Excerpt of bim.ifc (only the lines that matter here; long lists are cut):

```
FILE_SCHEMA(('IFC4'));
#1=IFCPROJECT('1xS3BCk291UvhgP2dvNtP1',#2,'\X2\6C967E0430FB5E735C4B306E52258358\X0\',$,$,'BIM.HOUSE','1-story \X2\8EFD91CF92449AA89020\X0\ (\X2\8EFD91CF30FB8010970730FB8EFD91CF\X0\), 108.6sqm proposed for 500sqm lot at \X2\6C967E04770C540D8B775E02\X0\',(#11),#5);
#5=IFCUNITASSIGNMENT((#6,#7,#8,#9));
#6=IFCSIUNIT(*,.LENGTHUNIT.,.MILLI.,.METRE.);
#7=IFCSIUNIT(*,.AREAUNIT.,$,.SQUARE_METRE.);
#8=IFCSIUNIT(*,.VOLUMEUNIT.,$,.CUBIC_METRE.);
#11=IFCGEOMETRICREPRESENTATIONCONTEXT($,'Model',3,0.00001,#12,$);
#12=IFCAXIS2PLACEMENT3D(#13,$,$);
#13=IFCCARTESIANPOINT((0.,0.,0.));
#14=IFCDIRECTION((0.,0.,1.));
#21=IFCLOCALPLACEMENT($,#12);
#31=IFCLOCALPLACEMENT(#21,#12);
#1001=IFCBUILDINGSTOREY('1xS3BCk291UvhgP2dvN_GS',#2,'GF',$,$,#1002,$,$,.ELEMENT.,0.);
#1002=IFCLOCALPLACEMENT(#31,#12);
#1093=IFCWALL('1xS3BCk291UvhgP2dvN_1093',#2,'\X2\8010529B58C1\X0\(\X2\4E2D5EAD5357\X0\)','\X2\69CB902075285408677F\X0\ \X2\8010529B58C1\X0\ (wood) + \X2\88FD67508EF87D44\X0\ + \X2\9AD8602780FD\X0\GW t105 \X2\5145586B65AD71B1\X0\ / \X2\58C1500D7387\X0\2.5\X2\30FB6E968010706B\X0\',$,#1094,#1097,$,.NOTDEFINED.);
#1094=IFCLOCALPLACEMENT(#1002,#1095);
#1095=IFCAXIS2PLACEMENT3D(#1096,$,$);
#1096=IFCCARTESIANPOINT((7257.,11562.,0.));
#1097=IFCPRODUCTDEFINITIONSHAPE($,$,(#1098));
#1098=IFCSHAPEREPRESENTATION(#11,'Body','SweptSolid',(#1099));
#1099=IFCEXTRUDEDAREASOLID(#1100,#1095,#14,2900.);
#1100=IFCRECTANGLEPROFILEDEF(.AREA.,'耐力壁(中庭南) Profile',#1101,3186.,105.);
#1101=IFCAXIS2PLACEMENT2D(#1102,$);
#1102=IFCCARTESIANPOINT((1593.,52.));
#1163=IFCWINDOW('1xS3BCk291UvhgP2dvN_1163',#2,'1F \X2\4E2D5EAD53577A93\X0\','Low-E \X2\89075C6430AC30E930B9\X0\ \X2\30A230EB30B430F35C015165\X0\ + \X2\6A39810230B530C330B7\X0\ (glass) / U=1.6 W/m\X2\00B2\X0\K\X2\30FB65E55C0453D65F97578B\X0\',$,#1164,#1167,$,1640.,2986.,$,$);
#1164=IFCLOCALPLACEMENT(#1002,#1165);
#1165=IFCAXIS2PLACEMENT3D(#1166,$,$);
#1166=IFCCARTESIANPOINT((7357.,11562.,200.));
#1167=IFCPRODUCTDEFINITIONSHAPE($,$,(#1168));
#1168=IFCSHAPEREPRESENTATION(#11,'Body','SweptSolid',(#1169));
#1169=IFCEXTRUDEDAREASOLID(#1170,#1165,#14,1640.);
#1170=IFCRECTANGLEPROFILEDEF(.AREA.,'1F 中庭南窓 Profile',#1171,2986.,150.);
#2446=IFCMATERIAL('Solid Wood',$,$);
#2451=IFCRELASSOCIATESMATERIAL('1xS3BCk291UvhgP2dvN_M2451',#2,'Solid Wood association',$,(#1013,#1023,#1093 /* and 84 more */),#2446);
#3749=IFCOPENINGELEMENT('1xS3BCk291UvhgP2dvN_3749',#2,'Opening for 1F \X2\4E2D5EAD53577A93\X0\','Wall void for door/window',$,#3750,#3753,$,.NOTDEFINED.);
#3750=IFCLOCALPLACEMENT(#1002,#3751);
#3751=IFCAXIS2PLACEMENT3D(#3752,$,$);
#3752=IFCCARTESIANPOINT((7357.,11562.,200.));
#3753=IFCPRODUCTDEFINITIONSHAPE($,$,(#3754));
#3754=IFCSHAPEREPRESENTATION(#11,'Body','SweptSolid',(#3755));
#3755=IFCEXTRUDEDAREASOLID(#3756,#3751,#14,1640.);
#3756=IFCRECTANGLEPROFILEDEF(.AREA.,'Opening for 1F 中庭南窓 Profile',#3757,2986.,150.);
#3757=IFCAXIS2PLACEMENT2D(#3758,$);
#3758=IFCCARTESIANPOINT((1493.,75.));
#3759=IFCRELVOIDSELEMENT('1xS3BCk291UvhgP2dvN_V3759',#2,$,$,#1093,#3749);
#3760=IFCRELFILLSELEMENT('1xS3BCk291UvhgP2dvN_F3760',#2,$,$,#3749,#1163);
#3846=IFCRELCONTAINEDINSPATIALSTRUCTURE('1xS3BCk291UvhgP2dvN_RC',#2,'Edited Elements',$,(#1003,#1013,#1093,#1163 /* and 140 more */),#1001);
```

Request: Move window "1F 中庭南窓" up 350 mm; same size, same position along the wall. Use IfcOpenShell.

```python
import numpy as np
import ifcopenshell
import ifcopenshell.api.geometry
import ifcopenshell.util.placement
import ifcopenshell.util.unit

model = ifcopenshell.open("bim.ifc")
unit_scale = ifcopenshell.util.unit.calculate_unit_scale(model)

window = model.by_guid("1xS3BCk291UvhgP2dvN_1163")
opening = window.FillsVoids[0].RelatingOpeningElement
dz = 0.35 / unit_scale

shift = np.array([0.0, 0.0, dz])
# The window is not placed relative to its opening, so move both.
for product in (opening, window):
    matrix = ifcopenshell.util.placement.get_local_placement(product.ObjectPlacement)
    matrix[:3, 3] += shift
    ifcopenshell.api.geometry.edit_object_placement(model, product=product, matrix=matrix, is_si=False)

print(f"moved by {dz * unit_scale:+.3f} m")

model.write("bim_updated.ifc")
```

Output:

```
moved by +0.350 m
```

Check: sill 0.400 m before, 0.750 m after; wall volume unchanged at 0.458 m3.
